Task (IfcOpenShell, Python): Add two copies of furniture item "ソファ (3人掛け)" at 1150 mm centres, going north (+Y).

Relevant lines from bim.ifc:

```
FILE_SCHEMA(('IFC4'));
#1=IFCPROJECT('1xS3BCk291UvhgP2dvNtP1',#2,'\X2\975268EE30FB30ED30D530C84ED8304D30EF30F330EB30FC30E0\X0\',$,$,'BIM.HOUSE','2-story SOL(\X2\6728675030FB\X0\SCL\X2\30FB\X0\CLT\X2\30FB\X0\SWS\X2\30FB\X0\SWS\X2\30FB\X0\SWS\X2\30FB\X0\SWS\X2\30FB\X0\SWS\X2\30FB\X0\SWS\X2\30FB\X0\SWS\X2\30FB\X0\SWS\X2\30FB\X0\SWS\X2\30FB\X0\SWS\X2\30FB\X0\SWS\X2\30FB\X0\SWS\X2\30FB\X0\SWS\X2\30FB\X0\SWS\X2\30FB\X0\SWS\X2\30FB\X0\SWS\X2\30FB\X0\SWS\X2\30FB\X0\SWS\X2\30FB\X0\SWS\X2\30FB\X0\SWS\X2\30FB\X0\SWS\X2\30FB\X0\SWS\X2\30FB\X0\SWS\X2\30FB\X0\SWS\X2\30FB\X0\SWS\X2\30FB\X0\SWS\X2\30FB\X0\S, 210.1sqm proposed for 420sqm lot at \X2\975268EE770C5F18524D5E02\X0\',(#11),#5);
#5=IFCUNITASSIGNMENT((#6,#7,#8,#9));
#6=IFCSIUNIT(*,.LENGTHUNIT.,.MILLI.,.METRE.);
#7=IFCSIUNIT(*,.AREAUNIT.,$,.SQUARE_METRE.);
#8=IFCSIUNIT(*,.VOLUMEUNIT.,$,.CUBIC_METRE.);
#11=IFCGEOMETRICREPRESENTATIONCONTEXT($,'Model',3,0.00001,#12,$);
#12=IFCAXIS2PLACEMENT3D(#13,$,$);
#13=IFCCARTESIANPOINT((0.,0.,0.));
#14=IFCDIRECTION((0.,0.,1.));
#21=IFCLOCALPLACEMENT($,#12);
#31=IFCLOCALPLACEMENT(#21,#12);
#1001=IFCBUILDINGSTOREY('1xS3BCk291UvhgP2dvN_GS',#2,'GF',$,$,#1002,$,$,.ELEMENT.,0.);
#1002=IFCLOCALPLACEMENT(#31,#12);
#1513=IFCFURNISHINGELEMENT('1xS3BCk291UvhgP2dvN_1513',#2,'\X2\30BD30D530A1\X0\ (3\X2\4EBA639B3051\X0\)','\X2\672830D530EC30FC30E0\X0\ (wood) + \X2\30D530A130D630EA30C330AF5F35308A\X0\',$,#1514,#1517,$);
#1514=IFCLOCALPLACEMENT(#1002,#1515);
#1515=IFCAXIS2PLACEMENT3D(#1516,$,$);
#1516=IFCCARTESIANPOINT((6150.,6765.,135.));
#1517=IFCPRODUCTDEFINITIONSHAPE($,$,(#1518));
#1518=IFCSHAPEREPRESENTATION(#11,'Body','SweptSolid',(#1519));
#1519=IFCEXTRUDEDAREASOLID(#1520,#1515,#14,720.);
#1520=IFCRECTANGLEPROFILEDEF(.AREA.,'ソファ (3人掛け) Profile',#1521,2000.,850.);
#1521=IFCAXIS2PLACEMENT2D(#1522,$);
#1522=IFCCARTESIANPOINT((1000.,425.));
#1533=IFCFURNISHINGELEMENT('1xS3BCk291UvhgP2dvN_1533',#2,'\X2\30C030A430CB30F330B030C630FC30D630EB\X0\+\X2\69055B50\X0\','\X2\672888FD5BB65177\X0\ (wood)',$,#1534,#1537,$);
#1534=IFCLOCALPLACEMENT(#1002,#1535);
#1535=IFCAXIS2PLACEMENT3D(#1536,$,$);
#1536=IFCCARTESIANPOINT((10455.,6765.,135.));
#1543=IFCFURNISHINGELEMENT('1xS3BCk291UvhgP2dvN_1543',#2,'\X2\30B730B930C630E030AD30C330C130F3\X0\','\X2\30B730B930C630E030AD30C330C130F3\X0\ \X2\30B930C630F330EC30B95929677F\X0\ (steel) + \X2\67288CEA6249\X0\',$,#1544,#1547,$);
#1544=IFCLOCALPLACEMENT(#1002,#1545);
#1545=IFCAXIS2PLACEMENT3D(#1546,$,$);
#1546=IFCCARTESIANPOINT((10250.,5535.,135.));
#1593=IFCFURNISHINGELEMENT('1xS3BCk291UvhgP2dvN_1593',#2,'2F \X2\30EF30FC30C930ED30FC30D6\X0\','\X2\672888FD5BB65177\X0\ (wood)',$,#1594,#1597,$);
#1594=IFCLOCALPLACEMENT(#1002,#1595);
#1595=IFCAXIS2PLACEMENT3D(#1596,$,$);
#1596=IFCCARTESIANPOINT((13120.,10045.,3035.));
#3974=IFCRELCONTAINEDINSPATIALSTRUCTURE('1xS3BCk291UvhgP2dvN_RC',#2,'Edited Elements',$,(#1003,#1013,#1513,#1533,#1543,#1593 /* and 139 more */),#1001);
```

```python
import numpy as np
import ifcopenshell
import ifcopenshell.api.geometry
import ifcopenshell.api.root
import ifcopenshell.util.element
import ifcopenshell.util.placement
import ifcopenshell.util.unit

model = ifcopenshell.open("bim.ifc")
unit_scale = ifcopenshell.util.unit.calculate_unit_scale(model)


def reuse_history(source, copy):
    """copy_class also copies each property set's owner history, people and application; keep the originals."""
    for rel in copy.IsDefinedBy:
        if rel.is_a("IfcRelDefinesByProperties") and (history := rel.RelatingPropertyDefinition.OwnerHistory):
            rel.RelatingPropertyDefinition.OwnerHistory = source.OwnerHistory
            ifcopenshell.util.element.remove_deep2(model, history)


source = model.by_guid("1xS3BCk291UvhgP2dvN_1513")
base = ifcopenshell.util.placement.get_local_placement(source.ObjectPlacement)
step = np.array([0.0, 1.0, 0.0]) * 1.15 / unit_scale

for i in range(1, 3):
    copy = ifcopenshell.api.root.copy_class(model, product=source)
    copy.Representation = ifcopenshell.util.element.copy_deep(
        model, source.Representation, exclude=["IfcGeometricRepresentationContext", "IfcRepresentationMap"]
    )
    reuse_history(source, copy)
    matrix = base.copy()
    matrix[:3, 3] += i * step
    print("added at", matrix[:3, 3].round(3) + 0.0)
    ifcopenshell.api.geometry.edit_object_placement(model, product=copy, matrix=matrix, is_si=False)

model.write("bim_updated.ifc")
```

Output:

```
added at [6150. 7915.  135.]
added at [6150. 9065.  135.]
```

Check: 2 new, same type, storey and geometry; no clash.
